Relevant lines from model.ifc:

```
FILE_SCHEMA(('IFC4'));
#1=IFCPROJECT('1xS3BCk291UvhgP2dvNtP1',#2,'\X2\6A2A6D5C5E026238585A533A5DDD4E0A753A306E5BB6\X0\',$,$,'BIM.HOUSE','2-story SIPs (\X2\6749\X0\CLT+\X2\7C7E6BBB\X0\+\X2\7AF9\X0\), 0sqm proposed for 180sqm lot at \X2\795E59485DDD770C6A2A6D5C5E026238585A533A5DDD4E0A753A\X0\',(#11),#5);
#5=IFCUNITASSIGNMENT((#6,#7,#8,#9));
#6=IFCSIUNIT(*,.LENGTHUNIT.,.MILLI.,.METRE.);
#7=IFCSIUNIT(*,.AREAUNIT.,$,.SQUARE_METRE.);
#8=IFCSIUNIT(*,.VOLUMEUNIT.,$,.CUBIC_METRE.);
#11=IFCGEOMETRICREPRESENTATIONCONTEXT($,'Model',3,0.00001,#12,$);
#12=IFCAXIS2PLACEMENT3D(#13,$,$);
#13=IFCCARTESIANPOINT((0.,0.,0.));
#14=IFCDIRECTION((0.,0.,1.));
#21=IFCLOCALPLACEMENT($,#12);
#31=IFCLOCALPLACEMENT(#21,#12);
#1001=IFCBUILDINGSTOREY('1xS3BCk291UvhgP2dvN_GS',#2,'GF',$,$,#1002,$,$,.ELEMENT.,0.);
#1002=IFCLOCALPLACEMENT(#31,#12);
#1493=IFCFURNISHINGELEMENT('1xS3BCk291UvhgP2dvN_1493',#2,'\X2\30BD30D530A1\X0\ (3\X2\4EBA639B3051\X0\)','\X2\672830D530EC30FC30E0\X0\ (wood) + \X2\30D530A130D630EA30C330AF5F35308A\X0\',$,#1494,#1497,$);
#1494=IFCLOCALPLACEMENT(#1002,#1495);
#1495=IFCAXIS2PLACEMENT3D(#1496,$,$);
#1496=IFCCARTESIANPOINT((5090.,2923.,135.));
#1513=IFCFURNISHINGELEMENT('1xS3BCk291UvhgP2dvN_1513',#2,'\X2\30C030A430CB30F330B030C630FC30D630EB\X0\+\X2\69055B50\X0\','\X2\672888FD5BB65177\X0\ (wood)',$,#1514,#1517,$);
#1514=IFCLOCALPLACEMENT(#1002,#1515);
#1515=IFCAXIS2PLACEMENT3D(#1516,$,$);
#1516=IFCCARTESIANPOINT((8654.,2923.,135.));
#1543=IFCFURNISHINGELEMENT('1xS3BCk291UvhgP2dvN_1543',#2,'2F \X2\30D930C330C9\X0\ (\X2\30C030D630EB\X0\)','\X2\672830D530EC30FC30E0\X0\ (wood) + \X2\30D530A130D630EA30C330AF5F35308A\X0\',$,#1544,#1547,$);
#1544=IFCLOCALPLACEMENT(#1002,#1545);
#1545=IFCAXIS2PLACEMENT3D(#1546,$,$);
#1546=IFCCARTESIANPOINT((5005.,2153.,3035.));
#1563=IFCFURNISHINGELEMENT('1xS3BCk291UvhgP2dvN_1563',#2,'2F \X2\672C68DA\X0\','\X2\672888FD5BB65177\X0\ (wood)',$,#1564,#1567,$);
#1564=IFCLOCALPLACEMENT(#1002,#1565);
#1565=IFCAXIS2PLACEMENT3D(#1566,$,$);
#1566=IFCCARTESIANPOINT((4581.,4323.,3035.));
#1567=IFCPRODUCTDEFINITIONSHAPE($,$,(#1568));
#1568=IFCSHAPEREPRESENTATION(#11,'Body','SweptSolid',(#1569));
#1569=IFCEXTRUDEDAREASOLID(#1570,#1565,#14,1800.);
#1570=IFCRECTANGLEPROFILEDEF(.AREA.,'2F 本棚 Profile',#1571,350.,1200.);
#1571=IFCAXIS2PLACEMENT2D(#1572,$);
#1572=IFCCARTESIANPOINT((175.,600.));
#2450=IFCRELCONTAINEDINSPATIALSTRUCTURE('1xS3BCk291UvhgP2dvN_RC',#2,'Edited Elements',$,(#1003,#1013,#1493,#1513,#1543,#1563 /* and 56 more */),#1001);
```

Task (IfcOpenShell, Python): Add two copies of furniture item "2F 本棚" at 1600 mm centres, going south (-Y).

```python
import numpy as np
import ifcopenshell
import ifcopenshell.api.geometry
import ifcopenshell.api.root
import ifcopenshell.util.element
import ifcopenshell.util.placement
import ifcopenshell.util.unit

model = ifcopenshell.open("model.ifc")
unit_scale = ifcopenshell.util.unit.calculate_unit_scale(model)


def reuse_history(source, copy):
    """copy_class also copies each property set's owner history, people and application; keep the originals."""
    for rel in copy.IsDefinedBy:
        if rel.is_a("IfcRelDefinesByProperties") and (history := rel.RelatingPropertyDefinition.OwnerHistory):
            rel.RelatingPropertyDefinition.OwnerHistory = source.OwnerHistory
            ifcopenshell.util.element.remove_deep2(model, history)


source = model.by_id(1563)
base = ifcopenshell.util.placement.get_local_placement(source.ObjectPlacement)
step = np.array([0.0, -1.0, 0.0]) * 1.6 / unit_scale

for i in range(1, 3):
    copy = ifcopenshell.api.root.copy_class(model, product=source)
    copy.Representation = ifcopenshell.util.element.copy_deep(
        model, source.Representation, exclude=["IfcGeometricRepresentationContext", "IfcRepresentationMap"]
    )
    reuse_history(source, copy)
    matrix = base.copy()
    matrix[:3, 3] += i * step
    print("added at", matrix[:3, 3].round(3) + 0.0)
    ifcopenshell.api.geometry.edit_object_placement(model, product=copy, matrix=matrix, is_si=False)

model.write("model_edited.ifc")
```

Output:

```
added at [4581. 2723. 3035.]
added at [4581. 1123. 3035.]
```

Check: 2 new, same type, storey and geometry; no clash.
